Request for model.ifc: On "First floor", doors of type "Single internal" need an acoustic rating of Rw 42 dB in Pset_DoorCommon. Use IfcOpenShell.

First a look at what the model holds.

```python
import ifcopenshell
import ifcopenshell.util.element

model = ifcopenshell.open("model.ifc")
print(model.schema)
storey = next(s for s in model.by_type("IfcBuildingStorey") if s.Name == "First floor")
doors = [e for e in ifcopenshell.util.element.get_decomposition(storey) if e.is_a("IfcDoor")]
seen = {}
for e in doors:
    element_type = ifcopenshell.util.element.get_type(e)
    key = (element_type.Name if element_type != e and element_type else None, ifcopenshell.util.element.get_pset(e, "Pset_DoorCommon", "AcousticRating"))
    seen[key] = seen.get(key, 0) + 1
for (name, value), count in sorted(seen.items(), key=str):
    print(count, "x", name, "|", value)
```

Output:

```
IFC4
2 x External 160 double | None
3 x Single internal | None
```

```python
import ifcopenshell
import ifcopenshell.api.pset
import ifcopenshell.util.element

model = ifcopenshell.open("model.ifc")

storey = next(s for s in model.by_type("IfcBuildingStorey") if s.Name == "First floor")
doors = [e for e in ifcopenshell.util.element.get_decomposition(storey) if e.is_a("IfcDoor")]

count = 0
for e in doors:
    element_type = ifcopenshell.util.element.get_type(e)
    if element_type in (None, e) or element_type.Name != "Single internal":
        continue
    # add_pset returns the element's existing set when there is one.
    pset = ifcopenshell.api.pset.add_pset(model, product=e, name="Pset_DoorCommon")
    ifcopenshell.api.pset.edit_pset(model, pset=pset, properties={"AcousticRating": "Rw 42 dB"})
    count += 1

print(count, "doors updated")

model.write("model_rev.ifc")
```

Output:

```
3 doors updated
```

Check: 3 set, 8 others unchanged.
